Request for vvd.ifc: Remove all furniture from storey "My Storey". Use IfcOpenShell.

First a look at what the model holds.

```python
import ifcopenshell
import ifcopenshell.util.element

model = ifcopenshell.open("vvd.ifc")
print(model.schema)
storey = next(s for s in model.by_type("IfcBuildingStorey") if s.Name == "My Storey")
furniture = [e for e in ifcopenshell.util.element.get_decomposition(storey) if e.is_a("IfcFurnishingElement")]
seen = {}
for e in furniture:
    element_type = ifcopenshell.util.element.get_type(e)
    name = element_type.Name if element_type not in (None, e) else None
    seen[name] = seen.get(name, 0) + 1
for name, count in sorted(seen.items(), key=str):
    print(count, "x", name)
```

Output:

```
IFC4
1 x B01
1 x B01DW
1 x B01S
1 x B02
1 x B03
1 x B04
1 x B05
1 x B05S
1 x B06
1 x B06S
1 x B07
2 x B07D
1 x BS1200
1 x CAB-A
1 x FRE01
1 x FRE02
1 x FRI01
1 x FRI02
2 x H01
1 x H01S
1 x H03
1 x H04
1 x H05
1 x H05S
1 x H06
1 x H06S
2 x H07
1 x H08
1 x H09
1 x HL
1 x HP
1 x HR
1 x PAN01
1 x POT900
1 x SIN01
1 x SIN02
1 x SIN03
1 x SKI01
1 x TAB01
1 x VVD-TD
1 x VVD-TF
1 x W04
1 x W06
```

```python
import ifcopenshell
import ifcopenshell.api.root
import ifcopenshell.util.element

model = ifcopenshell.open("vvd.ifc")

storey = next(s for s in model.by_type("IfcBuildingStorey") if s.Name == "My Storey")
furniture = [e for e in ifcopenshell.util.element.get_decomposition(storey) if e.is_a("IfcFurnishingElement")]

for e in furniture:
    ifcopenshell.api.root.remove_product(model, product=e)
print(len(furniture), "removed")

model.write("vvd_updated.ifc")
```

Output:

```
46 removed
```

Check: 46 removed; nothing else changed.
